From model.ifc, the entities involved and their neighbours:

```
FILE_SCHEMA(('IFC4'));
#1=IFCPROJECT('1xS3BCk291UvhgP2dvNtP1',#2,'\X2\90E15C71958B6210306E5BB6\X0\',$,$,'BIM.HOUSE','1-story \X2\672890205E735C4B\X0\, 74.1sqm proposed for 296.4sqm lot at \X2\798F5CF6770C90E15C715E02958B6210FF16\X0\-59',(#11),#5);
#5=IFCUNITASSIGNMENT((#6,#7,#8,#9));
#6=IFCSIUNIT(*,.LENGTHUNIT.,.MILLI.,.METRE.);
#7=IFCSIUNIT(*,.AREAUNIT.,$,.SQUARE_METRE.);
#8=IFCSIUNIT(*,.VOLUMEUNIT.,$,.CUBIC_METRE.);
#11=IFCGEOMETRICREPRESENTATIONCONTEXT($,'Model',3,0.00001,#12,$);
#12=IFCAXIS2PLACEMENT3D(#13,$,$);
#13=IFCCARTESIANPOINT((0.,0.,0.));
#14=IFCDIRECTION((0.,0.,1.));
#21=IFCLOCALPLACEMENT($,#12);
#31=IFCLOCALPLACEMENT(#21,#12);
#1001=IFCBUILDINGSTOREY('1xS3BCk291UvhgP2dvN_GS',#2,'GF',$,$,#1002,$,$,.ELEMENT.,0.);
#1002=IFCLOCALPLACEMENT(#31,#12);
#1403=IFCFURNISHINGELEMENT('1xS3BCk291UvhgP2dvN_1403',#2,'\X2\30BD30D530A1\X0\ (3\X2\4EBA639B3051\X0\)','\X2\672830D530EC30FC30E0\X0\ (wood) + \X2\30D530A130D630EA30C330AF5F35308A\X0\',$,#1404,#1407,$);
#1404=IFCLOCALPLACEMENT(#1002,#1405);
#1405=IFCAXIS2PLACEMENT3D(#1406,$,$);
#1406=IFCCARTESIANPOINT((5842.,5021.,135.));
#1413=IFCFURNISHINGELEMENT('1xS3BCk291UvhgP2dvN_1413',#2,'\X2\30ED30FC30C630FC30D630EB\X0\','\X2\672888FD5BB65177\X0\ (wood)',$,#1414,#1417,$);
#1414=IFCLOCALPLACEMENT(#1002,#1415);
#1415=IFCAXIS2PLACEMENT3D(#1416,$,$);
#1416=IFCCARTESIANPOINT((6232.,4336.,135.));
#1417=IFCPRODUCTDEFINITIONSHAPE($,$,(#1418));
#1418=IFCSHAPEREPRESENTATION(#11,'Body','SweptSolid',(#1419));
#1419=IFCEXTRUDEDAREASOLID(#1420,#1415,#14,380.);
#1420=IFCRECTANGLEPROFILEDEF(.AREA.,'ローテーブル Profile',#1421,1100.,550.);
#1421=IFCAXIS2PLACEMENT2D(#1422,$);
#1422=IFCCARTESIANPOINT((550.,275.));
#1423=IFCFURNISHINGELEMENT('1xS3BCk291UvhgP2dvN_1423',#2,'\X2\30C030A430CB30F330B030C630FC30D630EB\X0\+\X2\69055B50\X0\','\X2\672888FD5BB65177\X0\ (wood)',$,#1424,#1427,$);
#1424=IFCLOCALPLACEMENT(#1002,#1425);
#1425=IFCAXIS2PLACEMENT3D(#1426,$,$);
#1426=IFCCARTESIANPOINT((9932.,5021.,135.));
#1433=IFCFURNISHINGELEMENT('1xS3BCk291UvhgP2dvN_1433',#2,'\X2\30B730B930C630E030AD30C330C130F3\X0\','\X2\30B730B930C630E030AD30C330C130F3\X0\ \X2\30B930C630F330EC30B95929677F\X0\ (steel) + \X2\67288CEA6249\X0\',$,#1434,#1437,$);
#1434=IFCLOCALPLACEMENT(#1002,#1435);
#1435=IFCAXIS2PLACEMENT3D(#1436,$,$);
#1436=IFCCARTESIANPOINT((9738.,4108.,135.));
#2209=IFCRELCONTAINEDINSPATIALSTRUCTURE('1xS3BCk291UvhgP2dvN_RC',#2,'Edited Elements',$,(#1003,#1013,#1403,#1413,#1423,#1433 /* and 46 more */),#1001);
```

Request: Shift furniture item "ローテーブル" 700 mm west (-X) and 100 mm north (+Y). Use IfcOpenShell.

```python
import ifcopenshell
import ifcopenshell.api.geometry
import ifcopenshell.util.placement
import ifcopenshell.util.unit

model = ifcopenshell.open("model.ifc")
unit_scale = ifcopenshell.util.unit.calculate_unit_scale(model)

item = model.by_guid("1xS3BCk291UvhgP2dvN_1413")
matrix = ifcopenshell.util.placement.get_local_placement(item.ObjectPlacement)
matrix[0, 3] -= 0.7 / unit_scale
matrix[1, 3] += 0.1 / unit_scale
ifcopenshell.api.geometry.edit_object_placement(model, product=item, matrix=matrix, is_si=False)

print(ifcopenshell.util.placement.get_local_placement(item.ObjectPlacement).round(3) + 0.0)

model.write("model_v2.ifc")
```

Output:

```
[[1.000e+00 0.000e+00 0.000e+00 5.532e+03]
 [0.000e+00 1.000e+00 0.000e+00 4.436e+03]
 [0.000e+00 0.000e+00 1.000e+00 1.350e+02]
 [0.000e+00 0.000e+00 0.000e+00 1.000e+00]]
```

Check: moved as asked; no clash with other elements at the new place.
